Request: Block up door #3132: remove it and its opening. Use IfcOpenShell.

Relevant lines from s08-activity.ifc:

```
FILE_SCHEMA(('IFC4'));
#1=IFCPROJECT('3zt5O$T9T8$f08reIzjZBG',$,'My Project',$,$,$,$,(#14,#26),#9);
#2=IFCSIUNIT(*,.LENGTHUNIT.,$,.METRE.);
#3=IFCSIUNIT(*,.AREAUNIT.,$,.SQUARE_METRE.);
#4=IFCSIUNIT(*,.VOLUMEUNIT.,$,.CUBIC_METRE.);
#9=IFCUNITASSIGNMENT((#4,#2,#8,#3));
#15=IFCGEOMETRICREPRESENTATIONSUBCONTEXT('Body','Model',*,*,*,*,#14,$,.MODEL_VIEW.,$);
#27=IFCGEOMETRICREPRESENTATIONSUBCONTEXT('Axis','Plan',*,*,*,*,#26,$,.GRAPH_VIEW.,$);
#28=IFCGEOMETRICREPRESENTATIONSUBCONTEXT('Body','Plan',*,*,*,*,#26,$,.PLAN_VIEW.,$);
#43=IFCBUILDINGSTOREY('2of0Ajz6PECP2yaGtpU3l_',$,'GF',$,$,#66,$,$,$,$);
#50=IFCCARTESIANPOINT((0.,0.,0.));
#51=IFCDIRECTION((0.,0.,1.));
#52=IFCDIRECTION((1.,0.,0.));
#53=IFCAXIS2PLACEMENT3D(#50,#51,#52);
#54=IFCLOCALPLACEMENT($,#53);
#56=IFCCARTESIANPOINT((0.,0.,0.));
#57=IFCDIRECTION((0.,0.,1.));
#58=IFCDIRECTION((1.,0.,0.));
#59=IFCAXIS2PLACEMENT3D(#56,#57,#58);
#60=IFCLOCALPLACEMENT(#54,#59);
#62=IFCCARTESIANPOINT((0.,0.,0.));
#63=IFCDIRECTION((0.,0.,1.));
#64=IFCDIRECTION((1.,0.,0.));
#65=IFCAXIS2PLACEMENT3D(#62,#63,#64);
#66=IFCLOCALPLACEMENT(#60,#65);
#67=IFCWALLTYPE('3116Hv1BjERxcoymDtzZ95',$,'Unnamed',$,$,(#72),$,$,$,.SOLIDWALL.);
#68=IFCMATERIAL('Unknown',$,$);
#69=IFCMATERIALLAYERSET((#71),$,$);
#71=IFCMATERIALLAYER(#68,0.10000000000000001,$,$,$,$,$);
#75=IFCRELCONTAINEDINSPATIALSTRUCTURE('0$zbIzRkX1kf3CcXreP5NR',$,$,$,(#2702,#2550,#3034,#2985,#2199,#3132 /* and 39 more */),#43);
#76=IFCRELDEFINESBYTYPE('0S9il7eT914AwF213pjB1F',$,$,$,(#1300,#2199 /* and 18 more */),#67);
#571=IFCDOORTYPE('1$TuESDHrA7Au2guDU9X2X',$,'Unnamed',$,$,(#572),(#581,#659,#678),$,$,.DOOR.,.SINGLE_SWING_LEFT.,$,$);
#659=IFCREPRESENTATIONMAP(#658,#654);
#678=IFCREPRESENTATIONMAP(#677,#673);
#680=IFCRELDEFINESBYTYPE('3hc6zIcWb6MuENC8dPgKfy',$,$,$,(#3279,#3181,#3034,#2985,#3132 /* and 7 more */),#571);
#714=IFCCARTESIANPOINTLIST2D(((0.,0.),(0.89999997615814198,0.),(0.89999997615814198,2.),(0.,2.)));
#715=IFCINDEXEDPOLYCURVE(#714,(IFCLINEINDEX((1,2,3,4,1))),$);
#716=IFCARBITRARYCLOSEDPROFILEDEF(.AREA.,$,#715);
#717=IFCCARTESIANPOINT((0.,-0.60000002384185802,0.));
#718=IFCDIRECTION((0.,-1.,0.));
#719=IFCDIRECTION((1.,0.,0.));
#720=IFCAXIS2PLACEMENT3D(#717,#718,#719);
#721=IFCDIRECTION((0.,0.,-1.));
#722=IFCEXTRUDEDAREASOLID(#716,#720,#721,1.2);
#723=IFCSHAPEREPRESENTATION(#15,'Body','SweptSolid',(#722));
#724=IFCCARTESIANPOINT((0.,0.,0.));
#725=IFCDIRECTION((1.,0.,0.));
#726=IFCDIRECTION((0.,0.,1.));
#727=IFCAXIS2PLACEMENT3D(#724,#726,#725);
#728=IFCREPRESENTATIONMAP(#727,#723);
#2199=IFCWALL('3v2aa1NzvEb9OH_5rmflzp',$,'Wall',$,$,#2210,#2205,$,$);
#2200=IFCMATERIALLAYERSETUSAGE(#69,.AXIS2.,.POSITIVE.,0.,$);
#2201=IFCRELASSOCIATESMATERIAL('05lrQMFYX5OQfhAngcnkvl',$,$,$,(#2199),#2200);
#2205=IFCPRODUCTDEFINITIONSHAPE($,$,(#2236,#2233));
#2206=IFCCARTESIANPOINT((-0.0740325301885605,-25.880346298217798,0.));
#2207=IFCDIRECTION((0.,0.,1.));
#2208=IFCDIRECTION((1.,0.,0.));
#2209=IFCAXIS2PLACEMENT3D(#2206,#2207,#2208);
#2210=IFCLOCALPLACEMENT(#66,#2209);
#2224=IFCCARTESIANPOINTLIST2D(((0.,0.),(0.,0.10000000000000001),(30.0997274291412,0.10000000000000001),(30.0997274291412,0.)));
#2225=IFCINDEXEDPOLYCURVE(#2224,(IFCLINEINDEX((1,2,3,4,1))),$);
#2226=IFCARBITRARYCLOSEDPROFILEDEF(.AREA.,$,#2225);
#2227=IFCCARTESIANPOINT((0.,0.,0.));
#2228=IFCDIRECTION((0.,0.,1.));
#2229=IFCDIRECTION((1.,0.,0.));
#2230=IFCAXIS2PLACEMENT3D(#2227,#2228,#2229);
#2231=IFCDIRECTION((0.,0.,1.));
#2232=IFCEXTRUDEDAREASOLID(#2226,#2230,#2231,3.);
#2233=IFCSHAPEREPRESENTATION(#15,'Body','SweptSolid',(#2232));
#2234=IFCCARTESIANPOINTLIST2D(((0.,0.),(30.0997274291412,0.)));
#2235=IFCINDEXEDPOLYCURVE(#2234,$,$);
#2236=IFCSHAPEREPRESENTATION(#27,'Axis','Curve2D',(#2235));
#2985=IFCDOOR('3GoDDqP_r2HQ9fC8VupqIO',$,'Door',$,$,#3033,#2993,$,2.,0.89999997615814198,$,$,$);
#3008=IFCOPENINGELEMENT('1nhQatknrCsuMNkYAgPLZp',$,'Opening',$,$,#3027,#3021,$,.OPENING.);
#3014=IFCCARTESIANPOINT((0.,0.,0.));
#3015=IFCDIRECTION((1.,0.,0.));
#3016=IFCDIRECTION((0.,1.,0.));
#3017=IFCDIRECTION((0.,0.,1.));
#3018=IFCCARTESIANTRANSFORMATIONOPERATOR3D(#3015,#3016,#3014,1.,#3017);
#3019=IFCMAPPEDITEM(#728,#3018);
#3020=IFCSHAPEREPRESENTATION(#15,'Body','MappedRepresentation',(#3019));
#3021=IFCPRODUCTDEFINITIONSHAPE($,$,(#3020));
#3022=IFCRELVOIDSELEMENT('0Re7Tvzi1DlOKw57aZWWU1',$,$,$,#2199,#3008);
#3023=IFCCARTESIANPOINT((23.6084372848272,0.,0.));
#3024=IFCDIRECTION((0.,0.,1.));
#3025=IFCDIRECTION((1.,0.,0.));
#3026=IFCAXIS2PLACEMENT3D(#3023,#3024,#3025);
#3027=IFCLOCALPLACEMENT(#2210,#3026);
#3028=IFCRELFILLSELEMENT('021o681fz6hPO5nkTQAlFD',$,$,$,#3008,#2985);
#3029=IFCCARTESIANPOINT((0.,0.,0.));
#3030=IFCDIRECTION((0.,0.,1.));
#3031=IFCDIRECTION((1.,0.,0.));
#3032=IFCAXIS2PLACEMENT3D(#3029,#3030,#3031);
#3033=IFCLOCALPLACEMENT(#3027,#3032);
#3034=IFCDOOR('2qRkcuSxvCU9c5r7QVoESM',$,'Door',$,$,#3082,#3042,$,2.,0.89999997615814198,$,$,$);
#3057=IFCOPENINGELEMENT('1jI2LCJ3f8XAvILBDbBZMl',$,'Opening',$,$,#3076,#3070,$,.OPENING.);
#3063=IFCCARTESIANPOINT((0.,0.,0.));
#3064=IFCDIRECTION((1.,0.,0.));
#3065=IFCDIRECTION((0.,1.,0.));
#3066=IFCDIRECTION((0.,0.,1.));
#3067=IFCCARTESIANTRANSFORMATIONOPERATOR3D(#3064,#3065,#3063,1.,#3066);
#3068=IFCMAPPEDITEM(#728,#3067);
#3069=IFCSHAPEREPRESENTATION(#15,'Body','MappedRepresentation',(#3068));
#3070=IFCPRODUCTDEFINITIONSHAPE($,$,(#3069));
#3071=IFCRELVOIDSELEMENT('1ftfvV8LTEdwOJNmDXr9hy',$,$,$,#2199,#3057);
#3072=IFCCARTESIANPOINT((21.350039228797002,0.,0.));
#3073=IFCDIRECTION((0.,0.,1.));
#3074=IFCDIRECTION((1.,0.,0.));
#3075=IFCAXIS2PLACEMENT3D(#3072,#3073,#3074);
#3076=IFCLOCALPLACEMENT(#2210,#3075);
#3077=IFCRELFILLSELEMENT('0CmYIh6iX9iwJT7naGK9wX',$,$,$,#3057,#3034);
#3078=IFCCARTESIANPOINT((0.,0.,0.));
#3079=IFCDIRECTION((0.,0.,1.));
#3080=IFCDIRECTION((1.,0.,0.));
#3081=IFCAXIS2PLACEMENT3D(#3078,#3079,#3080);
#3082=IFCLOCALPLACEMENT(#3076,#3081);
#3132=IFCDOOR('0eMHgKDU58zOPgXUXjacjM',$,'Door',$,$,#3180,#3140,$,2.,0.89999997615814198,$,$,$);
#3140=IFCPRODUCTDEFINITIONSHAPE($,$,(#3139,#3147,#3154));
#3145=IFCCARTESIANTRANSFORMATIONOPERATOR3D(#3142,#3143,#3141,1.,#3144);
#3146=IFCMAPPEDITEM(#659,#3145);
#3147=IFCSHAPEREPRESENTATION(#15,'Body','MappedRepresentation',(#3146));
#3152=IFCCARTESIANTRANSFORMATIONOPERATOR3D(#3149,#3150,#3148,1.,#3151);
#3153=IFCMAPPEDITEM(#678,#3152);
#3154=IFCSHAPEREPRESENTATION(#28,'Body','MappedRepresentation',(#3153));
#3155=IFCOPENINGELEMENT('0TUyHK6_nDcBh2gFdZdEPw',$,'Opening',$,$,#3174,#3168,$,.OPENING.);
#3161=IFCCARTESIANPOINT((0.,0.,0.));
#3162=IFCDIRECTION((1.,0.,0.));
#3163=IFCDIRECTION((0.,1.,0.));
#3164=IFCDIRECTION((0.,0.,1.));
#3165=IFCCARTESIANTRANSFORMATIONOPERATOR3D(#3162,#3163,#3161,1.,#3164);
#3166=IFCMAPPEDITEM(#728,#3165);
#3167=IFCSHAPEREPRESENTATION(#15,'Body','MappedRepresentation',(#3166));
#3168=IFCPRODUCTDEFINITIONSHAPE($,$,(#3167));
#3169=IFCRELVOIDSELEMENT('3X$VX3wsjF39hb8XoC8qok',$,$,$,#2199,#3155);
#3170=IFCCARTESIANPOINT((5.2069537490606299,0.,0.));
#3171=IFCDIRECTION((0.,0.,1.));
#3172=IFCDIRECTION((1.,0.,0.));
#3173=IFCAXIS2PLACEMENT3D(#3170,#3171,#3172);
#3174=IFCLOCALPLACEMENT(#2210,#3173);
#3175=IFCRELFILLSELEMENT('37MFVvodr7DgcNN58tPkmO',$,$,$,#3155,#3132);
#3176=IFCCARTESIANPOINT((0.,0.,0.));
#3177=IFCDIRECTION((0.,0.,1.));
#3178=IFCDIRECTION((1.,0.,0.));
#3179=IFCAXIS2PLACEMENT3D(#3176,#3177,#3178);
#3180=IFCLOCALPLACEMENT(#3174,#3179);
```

```python
import ifcopenshell
import ifcopenshell.api.feature
import ifcopenshell.api.root
import ifcopenshell.geom
import ifcopenshell.util.shape

model = ifcopenshell.open("s08-activity.ifc")
settings = ifcopenshell.geom.settings()


def volume(element):
    """Net volume in cubic metres, openings subtracted."""
    shape = ifcopenshell.geom.create_shape(settings, element)
    return ifcopenshell.util.shape.get_volume(shape.geometry)


door = model.by_id(3132)
opening = door.FillsVoids[0].RelatingOpeningElement
wall = opening.VoidsElements[0].RelatingBuildingElement
before = volume(wall)

ifcopenshell.api.root.remove_product(model, product=door)
ifcopenshell.api.feature.remove_feature(model, feature=opening)

after = volume(wall)

print(f"wall volume {before:.3f} -> {after:.3f} m3")

model.write("s08-activity-out.ifc")
```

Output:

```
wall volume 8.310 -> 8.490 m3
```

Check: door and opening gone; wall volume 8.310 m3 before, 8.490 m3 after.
